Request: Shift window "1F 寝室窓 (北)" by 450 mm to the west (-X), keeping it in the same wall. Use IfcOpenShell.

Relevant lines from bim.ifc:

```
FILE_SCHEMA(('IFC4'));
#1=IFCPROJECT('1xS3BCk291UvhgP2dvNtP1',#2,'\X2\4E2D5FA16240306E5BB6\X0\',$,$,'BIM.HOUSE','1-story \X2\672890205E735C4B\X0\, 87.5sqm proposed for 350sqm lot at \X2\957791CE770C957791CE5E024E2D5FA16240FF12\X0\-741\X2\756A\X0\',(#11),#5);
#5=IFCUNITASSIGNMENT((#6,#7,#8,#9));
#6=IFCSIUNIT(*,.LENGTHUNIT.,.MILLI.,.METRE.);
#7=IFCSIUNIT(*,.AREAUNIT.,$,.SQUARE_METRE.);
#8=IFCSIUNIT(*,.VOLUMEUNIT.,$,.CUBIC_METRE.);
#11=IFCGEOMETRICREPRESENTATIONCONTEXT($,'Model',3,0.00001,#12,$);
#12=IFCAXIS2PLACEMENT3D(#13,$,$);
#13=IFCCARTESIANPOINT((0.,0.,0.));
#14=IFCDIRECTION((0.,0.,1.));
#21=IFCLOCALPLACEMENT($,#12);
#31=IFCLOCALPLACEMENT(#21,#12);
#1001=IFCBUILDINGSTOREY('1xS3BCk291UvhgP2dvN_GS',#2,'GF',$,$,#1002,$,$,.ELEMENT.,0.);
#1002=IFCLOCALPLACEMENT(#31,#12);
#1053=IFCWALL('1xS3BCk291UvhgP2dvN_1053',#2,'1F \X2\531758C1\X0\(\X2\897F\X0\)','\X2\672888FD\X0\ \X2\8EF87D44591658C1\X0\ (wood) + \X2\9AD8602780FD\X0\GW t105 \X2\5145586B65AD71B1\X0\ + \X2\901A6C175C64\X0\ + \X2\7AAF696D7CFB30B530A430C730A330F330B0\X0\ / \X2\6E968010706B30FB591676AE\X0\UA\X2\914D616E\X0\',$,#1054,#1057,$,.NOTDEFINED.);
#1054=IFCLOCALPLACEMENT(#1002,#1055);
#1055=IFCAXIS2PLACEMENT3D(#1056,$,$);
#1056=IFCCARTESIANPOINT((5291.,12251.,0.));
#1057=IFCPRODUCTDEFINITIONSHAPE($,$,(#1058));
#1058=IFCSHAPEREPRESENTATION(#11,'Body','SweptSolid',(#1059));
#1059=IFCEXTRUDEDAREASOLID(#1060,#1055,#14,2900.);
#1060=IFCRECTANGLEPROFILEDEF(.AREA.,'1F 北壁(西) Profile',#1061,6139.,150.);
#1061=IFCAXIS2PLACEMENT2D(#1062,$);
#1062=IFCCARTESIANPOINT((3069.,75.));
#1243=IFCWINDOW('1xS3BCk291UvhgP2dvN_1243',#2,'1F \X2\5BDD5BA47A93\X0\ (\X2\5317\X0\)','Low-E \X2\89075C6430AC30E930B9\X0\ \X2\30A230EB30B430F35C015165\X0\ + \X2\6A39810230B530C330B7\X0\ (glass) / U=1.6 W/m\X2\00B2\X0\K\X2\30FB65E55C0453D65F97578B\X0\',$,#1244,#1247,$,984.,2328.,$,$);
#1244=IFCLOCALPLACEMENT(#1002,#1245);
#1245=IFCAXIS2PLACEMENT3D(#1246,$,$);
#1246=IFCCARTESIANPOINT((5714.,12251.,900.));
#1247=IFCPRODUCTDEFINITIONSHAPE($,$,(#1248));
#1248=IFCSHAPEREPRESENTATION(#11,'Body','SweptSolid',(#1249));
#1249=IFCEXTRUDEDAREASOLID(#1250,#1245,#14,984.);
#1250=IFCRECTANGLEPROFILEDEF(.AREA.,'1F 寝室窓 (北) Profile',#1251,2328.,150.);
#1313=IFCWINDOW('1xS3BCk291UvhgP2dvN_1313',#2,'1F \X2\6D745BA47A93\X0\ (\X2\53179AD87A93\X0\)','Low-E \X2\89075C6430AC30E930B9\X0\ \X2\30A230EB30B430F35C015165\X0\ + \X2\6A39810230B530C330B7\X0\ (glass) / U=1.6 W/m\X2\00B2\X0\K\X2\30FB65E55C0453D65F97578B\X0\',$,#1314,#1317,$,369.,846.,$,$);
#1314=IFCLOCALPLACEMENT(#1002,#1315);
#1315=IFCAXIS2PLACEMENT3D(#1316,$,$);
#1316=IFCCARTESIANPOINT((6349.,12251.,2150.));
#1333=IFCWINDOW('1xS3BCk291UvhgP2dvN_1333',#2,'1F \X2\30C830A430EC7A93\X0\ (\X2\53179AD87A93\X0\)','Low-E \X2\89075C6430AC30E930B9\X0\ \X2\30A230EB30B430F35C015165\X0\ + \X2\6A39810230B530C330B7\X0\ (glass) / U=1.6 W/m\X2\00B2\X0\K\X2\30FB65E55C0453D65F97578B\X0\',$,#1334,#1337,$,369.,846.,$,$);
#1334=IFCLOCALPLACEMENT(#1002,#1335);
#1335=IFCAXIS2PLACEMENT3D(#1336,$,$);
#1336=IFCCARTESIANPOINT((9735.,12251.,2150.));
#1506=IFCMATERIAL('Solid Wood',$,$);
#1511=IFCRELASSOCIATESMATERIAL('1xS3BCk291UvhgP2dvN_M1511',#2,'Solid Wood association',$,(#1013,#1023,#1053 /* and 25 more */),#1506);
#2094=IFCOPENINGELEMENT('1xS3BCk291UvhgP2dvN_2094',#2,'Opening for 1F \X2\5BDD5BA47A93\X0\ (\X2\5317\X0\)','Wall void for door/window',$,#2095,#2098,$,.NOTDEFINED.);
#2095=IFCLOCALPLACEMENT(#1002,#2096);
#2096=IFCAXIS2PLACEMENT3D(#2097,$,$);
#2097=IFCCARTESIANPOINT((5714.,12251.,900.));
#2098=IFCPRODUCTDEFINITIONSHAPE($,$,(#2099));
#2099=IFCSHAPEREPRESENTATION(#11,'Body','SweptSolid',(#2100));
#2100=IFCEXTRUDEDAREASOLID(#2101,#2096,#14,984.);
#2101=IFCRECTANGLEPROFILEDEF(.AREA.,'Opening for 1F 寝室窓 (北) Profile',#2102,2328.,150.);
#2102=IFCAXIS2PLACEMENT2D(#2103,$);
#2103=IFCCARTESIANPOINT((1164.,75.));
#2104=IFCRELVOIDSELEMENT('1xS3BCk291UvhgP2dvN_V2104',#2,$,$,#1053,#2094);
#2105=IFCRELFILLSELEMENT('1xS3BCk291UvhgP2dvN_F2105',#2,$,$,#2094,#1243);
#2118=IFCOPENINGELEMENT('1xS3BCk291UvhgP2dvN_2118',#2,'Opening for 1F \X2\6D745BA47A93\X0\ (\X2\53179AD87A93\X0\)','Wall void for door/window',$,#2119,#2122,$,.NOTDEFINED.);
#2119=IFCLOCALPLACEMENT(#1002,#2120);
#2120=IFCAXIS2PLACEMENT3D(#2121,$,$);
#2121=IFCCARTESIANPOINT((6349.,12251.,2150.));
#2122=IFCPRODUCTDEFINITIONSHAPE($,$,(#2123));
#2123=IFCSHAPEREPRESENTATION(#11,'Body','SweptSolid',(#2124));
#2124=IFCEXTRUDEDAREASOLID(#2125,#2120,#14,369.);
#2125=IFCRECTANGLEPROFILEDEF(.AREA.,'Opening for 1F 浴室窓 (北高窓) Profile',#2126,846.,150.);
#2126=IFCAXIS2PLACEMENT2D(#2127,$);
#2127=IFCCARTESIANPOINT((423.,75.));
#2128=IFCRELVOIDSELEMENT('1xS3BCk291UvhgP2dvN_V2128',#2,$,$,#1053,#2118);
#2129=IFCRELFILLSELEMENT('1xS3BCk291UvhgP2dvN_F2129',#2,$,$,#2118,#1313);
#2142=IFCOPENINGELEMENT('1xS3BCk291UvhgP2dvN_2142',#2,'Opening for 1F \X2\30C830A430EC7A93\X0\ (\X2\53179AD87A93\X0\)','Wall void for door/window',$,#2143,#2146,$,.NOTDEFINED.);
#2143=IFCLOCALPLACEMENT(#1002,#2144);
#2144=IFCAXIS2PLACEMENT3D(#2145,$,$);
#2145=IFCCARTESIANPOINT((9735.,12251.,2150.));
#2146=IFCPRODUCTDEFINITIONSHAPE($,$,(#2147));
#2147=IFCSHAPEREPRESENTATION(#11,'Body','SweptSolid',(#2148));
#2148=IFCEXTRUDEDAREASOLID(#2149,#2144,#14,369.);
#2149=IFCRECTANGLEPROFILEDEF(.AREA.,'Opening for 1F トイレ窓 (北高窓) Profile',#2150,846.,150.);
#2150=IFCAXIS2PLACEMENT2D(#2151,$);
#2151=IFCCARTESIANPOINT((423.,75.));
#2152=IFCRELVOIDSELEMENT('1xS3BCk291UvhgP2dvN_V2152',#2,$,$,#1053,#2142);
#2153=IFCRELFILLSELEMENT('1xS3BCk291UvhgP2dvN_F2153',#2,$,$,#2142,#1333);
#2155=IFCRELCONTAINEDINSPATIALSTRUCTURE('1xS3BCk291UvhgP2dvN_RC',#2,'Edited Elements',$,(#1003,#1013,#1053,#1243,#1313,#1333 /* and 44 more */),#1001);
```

```python
import ifcopenshell
import ifcopenshell.api.geometry
import ifcopenshell.util.placement

model = ifcopenshell.open("bim.ifc")

window = model.by_guid("1xS3BCk291UvhgP2dvN_1243")
opening = window.FillsVoids[0].RelatingOpeningElement
wall = opening.VoidsElements[0].RelatingBuildingElement

wall_matrix = ifcopenshell.util.placement.get_local_placement(wall.ObjectPlacement)
shift = wall_matrix[:3, 0] * -450.0
before = ifcopenshell.util.placement.get_local_placement(window.ObjectPlacement)[:3, 3].copy()

# The window is not placed relative to its opening, so move both.
for product in (opening, window):
    matrix = ifcopenshell.util.placement.get_local_placement(product.ObjectPlacement)
    matrix[:3, 3] += shift
    ifcopenshell.api.geometry.edit_object_placement(model, product=product, matrix=matrix, is_si=False)

after = ifcopenshell.util.placement.get_local_placement(window.ObjectPlacement)[:3, 3]
print("window moved by", (after - before).round(3) + 0.0)

model.write("bim_v2.ifc")
```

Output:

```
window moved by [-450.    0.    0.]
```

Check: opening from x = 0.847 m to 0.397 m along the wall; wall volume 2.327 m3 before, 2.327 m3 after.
